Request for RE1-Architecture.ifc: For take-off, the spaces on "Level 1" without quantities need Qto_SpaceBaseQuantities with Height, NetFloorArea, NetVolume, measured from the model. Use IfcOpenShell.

First a look at what the model holds.

```python
import ifcopenshell
import ifcopenshell.util.element
import ifcopenshell.util.unit

model = ifcopenshell.open("RE1-Architecture.ifc")
print(model.schema)
for unit_type in ("LENGTHUNIT", "AREAUNIT", "VOLUMEUNIT"):
    print(unit_type, ifcopenshell.util.unit.calculate_unit_scale(model, unit_type))
storey = next(s for s in model.by_type("IfcBuildingStorey") if s.Name == "Level 1")
spaces = [e for e in ifcopenshell.util.element.get_decomposition(storey) if e.is_a("IfcSpace")]
for e in sorted(spaces, key=lambda e: e.id()):
    print(e.id(), e.is_a(), e.Name, list(ifcopenshell.util.element.get_psets(e, qtos_only=True)), sep=" | ")
```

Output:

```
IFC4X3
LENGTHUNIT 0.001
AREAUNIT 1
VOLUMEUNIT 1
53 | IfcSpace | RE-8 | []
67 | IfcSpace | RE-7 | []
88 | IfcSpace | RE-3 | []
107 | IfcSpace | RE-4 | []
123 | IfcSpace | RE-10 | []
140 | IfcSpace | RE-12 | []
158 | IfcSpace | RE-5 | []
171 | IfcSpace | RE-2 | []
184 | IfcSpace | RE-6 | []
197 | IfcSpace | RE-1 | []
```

```python
import ifcopenshell
import ifcopenshell.api.pset
import ifcopenshell.geom
import ifcopenshell.util.element
import ifcopenshell.util.shape
import ifcopenshell.util.unit

model = ifcopenshell.open("RE1-Architecture.ifc")
unit_scale = ifcopenshell.util.unit.calculate_unit_scale(model)
area_scale = ifcopenshell.util.unit.calculate_unit_scale(model, "AREAUNIT")
volume_scale = ifcopenshell.util.unit.calculate_unit_scale(model, "VOLUMEUNIT")
settings = ifcopenshell.geom.settings()

storey = next(s for s in model.by_type("IfcBuildingStorey") if s.Name == "Level 1")
spaces = [e for e in ifcopenshell.util.element.get_decomposition(storey) if e.is_a("IfcSpace")]

for e in sorted(spaces, key=lambda e: e.id()):
    if ifcopenshell.util.element.get_psets(e, qtos_only=True, should_inherit=False):
        continue
    # Geometry comes back in metres, in the element's own axes.
    shape = ifcopenshell.geom.create_shape(settings, e)
    values = {
        "Height": ifcopenshell.util.shape.get_z(shape.geometry) / unit_scale,
        "NetFloorArea": ifcopenshell.util.shape.get_footprint_area(shape.geometry) / area_scale,
        "NetVolume": ifcopenshell.util.shape.get_volume(shape.geometry) / volume_scale,
    }
    qto = ifcopenshell.api.pset.add_qto(model, product=e, name="Qto_SpaceBaseQuantities")
    ifcopenshell.api.pset.edit_qto(model, qto=qto, properties=values)
    print(e.id(), {k: round(v, 3) for k, v in values.items()})

model.write("RE1-Architecture_v2.ifc")
```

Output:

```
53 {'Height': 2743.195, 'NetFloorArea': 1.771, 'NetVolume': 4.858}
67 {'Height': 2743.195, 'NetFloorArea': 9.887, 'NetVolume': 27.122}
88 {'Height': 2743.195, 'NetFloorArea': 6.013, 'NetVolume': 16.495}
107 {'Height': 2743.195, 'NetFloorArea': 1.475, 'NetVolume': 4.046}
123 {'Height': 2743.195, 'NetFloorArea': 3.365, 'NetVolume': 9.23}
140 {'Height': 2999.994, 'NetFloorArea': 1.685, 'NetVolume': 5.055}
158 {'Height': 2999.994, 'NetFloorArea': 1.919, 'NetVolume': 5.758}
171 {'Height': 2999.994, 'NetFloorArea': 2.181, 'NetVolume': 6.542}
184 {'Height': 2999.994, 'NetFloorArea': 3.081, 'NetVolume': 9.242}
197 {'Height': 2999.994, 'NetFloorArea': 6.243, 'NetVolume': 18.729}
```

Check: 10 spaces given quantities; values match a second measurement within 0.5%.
